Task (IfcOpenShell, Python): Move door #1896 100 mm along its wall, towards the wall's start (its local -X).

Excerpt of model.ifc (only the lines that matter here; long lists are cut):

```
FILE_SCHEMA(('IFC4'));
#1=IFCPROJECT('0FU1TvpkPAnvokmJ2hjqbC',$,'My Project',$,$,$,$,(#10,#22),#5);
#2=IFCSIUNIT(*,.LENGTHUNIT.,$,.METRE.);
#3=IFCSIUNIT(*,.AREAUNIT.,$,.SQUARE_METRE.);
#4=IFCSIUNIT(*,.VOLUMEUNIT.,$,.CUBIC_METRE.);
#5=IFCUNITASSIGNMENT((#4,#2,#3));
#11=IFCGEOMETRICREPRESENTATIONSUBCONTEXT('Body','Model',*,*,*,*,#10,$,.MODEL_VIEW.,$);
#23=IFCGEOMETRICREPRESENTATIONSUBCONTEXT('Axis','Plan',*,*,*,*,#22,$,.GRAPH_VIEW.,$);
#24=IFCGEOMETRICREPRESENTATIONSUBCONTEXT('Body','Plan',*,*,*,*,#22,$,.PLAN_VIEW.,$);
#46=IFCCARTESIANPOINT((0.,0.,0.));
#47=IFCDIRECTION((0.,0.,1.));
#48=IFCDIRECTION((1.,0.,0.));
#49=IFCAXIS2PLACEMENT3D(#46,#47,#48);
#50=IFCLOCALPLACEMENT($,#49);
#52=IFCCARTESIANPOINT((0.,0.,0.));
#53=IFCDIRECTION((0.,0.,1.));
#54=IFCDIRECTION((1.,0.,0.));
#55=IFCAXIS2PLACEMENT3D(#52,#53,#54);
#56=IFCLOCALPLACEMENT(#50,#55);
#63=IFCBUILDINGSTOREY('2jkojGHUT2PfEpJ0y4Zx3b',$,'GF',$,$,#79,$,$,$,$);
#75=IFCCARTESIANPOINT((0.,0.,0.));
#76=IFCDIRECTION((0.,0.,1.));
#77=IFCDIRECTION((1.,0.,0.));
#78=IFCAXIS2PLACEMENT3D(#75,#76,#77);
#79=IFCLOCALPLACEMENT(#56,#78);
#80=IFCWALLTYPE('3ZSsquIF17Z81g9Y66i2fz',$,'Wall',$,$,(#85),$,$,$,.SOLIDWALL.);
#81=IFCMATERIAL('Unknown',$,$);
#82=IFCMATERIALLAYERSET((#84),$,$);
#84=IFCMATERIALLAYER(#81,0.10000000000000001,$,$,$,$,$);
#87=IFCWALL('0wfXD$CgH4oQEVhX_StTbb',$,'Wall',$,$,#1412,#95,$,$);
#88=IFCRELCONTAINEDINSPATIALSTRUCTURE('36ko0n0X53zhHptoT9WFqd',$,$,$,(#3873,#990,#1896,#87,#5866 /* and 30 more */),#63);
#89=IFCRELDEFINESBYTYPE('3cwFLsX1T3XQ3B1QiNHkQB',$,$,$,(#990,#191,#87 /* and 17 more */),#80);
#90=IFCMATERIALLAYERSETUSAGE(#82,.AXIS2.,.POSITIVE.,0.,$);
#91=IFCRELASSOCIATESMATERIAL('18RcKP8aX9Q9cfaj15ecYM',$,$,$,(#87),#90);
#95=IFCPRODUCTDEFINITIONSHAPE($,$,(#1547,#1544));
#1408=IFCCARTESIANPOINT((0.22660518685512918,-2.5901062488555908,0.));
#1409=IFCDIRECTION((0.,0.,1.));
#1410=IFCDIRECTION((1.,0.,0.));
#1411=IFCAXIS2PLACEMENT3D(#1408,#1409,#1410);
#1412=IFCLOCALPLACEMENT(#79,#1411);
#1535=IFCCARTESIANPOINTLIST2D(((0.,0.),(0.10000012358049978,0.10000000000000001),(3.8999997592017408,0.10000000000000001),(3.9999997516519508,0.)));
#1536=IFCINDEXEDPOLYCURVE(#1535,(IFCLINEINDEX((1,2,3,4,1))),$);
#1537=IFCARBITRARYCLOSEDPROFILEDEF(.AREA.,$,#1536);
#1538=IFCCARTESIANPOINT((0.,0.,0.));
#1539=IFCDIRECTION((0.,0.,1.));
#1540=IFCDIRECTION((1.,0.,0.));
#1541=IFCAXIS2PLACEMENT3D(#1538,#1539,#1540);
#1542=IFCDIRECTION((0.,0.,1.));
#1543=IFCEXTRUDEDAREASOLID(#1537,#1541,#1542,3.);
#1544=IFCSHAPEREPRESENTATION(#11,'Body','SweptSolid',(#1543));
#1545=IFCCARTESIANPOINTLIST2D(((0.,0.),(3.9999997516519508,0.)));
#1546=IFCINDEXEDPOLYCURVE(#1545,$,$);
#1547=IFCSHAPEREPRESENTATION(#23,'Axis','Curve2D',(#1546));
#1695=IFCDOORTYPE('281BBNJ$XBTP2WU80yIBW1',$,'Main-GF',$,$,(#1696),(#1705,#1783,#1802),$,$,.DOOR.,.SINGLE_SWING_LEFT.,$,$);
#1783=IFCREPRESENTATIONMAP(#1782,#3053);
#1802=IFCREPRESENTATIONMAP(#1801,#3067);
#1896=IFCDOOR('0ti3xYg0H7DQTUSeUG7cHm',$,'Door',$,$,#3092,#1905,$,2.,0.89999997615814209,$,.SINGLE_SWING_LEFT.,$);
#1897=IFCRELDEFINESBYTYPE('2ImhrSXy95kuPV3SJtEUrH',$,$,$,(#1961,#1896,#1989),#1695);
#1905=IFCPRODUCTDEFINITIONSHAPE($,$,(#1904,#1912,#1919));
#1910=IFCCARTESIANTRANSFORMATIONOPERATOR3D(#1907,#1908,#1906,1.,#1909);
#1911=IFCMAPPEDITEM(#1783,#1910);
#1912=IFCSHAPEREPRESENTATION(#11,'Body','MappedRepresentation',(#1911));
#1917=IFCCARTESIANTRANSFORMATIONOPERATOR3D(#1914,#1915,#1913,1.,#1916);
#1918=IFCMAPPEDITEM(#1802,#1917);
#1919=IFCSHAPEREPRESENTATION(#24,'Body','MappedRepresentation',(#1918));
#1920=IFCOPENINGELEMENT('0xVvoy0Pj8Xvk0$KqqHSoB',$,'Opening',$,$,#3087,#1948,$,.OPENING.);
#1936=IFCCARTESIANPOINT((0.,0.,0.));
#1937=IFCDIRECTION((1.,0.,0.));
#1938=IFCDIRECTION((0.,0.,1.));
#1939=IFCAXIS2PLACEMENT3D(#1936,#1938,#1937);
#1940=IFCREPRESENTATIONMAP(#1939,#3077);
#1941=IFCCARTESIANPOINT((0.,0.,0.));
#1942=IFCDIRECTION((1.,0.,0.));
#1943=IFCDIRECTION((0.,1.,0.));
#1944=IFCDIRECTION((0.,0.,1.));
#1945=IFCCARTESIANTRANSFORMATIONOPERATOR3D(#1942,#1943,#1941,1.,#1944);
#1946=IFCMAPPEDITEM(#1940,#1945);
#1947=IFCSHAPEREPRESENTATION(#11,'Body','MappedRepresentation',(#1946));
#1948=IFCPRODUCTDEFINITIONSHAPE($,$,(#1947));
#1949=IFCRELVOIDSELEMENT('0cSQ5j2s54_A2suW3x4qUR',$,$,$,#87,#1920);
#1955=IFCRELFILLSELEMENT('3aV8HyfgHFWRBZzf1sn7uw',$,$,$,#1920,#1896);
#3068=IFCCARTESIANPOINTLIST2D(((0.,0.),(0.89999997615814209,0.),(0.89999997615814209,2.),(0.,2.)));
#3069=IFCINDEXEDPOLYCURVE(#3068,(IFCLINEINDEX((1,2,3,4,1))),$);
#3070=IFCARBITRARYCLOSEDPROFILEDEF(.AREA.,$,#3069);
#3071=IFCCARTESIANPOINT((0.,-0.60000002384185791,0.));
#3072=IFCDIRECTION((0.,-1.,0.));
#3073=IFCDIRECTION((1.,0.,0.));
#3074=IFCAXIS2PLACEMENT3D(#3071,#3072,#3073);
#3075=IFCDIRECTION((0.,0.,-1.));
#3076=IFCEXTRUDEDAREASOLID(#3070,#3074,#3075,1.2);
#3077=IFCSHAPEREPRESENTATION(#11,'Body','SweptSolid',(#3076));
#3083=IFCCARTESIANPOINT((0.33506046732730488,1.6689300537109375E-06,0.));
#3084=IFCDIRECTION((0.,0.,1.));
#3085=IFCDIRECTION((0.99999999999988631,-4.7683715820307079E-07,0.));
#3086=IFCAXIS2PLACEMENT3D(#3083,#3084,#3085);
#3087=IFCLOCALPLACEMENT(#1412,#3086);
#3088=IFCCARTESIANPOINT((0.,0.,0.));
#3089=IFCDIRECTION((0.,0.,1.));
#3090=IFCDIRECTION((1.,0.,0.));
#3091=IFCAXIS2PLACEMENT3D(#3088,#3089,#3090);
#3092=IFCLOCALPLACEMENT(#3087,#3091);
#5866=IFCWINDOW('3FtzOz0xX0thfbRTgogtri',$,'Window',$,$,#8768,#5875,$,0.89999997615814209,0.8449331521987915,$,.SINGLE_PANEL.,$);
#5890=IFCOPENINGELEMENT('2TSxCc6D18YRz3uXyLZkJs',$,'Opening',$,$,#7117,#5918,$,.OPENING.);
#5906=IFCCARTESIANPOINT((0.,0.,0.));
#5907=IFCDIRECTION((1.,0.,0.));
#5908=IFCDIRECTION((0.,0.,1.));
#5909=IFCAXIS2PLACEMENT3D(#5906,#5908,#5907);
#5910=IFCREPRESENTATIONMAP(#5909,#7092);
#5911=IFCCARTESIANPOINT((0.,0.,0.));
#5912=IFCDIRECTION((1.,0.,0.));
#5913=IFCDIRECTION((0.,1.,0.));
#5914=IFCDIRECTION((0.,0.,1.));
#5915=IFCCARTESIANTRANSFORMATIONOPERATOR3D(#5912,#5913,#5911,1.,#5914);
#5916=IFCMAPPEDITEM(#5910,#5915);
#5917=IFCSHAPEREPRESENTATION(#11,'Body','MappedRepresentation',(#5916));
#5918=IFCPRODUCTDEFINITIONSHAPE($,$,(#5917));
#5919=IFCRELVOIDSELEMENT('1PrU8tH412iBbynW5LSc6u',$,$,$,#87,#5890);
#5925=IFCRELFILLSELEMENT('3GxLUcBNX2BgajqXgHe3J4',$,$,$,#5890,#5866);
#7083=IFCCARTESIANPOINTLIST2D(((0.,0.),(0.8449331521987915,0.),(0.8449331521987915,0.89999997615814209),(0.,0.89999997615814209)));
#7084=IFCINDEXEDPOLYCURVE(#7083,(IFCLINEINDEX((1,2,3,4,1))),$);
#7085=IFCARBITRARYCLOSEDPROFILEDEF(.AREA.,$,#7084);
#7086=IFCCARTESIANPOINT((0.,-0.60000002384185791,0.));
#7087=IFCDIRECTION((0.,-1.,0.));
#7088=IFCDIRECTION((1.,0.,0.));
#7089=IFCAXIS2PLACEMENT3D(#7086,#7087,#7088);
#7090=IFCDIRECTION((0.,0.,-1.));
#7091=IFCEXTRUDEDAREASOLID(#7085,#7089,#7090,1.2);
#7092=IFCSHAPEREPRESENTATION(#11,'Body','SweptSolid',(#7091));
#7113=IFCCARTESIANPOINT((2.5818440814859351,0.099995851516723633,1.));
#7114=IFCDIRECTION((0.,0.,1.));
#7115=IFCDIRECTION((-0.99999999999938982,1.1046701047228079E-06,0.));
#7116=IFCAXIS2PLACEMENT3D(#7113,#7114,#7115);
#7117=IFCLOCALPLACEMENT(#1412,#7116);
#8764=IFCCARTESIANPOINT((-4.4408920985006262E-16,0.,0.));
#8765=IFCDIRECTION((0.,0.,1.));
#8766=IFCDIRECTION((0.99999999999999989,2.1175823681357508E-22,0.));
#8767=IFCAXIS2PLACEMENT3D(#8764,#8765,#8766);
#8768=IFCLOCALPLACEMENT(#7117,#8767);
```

```python
import ifcopenshell
import ifcopenshell.api.geometry
import ifcopenshell.util.placement

model = ifcopenshell.open("model.ifc")

door = model.by_guid("0ti3xYg0H7DQTUSeUG7cHm")
opening = door.FillsVoids[0].RelatingOpeningElement
wall = opening.VoidsElements[0].RelatingBuildingElement

wall_matrix = ifcopenshell.util.placement.get_local_placement(wall.ObjectPlacement)
shift = wall_matrix[:3, 0] * -0.1
before = ifcopenshell.util.placement.get_local_placement(door.ObjectPlacement)[:3, 3].copy()

# The door is placed relative to its opening, so it follows when the opening moves.
matrix = ifcopenshell.util.placement.get_local_placement(opening.ObjectPlacement)
matrix[:3, 3] += shift
ifcopenshell.api.geometry.edit_object_placement(
    model, product=opening, matrix=matrix, is_si=False, should_transform_children=True
)

after = ifcopenshell.util.placement.get_local_placement(door.ObjectPlacement)[:3, 3]
print("door moved by", (after - before).round(3) + 0.0)

model.write("model_rev.ifc")
```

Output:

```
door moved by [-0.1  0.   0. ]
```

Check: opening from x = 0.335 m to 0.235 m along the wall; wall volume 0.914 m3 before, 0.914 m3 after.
